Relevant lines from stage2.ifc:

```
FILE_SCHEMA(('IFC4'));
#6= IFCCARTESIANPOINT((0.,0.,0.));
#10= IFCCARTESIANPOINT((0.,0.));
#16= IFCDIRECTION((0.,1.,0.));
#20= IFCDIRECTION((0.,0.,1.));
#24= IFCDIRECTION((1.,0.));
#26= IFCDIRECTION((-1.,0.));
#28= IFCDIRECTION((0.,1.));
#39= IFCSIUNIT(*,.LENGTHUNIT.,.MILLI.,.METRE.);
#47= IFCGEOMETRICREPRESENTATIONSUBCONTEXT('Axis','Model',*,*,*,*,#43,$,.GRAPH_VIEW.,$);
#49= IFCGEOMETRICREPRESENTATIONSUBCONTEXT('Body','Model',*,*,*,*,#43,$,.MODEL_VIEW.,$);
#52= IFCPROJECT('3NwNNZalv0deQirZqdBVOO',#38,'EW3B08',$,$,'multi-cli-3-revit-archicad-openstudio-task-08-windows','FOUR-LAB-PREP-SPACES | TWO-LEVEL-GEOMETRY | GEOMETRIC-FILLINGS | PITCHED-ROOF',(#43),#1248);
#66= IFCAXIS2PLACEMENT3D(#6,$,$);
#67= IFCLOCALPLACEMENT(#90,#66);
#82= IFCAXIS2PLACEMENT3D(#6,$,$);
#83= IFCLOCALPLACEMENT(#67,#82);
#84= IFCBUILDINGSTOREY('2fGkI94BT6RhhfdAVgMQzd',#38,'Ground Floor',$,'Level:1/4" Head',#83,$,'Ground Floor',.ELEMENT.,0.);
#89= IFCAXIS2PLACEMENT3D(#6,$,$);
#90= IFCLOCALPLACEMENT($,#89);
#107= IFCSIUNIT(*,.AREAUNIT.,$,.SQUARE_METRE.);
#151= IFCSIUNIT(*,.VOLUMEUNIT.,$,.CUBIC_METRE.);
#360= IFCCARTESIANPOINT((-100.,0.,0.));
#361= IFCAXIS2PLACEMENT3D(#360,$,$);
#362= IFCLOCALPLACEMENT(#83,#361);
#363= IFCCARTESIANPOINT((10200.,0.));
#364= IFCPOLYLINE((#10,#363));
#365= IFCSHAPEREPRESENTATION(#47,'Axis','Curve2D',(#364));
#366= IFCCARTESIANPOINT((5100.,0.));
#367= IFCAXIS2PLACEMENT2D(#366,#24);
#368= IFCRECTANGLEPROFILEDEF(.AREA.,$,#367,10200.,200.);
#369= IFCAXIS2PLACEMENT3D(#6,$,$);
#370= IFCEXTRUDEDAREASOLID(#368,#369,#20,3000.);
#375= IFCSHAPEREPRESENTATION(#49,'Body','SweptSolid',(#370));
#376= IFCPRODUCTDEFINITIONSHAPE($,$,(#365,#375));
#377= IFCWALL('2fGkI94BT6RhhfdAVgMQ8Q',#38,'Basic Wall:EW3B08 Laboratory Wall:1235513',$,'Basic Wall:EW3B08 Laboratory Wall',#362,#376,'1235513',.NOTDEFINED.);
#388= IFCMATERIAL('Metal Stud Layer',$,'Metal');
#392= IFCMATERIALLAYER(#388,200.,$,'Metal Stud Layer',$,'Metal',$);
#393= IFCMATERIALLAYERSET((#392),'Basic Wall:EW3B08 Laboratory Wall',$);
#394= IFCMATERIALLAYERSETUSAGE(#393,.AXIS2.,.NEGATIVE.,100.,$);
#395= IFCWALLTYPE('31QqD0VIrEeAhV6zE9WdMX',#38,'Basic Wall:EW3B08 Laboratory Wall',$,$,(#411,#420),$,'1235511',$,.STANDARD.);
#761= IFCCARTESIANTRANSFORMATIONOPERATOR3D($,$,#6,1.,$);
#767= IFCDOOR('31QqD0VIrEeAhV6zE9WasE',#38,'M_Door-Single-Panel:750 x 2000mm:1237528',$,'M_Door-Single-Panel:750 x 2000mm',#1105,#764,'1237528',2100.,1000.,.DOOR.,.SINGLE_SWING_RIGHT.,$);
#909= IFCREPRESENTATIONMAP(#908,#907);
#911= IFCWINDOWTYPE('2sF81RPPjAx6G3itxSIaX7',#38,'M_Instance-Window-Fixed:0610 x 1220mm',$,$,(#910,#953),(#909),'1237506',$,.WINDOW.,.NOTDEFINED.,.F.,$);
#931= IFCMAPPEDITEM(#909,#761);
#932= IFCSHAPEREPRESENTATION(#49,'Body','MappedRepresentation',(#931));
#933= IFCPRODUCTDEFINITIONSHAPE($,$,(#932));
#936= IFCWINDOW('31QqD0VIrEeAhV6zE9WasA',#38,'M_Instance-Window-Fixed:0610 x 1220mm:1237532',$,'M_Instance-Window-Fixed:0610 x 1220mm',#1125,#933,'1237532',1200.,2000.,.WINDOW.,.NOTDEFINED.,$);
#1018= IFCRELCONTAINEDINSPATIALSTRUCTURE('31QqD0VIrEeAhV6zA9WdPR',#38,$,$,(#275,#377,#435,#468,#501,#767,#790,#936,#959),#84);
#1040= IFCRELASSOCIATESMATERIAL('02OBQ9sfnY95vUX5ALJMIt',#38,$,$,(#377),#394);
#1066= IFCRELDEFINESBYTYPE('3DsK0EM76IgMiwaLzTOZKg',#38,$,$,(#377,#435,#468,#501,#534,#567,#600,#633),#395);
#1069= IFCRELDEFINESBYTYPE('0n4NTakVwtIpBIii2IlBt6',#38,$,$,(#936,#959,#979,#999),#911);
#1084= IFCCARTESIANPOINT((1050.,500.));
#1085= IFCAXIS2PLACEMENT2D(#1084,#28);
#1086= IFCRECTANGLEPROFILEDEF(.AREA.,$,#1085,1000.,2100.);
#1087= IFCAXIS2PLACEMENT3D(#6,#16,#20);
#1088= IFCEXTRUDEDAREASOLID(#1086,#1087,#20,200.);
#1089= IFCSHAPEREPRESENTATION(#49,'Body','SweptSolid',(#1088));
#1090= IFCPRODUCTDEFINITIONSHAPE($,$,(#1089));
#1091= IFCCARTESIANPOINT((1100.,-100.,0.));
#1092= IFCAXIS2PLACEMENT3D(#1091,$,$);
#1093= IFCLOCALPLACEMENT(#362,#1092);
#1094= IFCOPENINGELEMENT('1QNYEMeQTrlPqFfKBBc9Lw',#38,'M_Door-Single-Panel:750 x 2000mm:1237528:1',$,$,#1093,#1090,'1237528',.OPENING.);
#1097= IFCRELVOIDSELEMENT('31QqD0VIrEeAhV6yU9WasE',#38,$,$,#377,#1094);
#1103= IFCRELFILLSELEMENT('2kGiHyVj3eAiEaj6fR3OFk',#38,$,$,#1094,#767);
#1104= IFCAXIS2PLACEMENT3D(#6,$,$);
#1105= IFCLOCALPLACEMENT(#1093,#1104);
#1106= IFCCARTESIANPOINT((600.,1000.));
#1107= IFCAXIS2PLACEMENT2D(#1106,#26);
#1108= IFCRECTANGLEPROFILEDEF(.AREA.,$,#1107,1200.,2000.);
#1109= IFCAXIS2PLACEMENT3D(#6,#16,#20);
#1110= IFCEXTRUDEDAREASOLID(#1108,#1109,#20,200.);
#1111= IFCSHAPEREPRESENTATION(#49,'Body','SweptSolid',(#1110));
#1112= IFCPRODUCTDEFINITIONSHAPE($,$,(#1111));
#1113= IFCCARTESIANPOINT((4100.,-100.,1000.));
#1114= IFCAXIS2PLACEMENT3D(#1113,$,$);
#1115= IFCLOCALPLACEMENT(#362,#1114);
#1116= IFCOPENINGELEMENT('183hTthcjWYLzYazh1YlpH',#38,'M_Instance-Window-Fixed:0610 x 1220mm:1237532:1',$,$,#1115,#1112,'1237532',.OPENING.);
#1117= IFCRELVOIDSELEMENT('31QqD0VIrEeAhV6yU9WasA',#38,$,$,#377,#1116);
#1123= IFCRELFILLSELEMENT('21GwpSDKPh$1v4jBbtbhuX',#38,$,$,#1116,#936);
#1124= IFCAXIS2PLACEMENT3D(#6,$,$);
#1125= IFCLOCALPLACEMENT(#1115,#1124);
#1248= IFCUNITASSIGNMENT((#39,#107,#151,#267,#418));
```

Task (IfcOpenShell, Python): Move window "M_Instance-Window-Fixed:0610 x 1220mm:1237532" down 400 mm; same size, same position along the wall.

```python
import numpy as np
import ifcopenshell
import ifcopenshell.api.geometry
import ifcopenshell.util.placement
import ifcopenshell.util.unit

model = ifcopenshell.open("stage2.ifc")
unit_scale = ifcopenshell.util.unit.calculate_unit_scale(model)

window = model.by_guid("31QqD0VIrEeAhV6zE9WasA")
opening = window.FillsVoids[0].RelatingOpeningElement
dz = -400.0

shift = np.array([0.0, 0.0, dz])
# The window is placed relative to its opening, so it follows when the opening moves.
matrix = ifcopenshell.util.placement.get_local_placement(opening.ObjectPlacement)
matrix[:3, 3] += shift
ifcopenshell.api.geometry.edit_object_placement(
    model, product=opening, matrix=matrix, is_si=False, should_transform_children=True
)

print(f"moved by {dz * unit_scale:+.3f} m")

model.write("stage2_rev.ifc")
```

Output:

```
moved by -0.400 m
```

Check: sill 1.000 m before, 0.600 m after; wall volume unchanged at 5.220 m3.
